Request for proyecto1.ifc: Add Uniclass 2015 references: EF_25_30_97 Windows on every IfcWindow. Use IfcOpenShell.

First a look at what the model holds.

```python
import ifcopenshell

model = ifcopenshell.open("proyecto1.ifc")
print(model.schema)
print("classifications:", [c.Name for c in model.by_type("IfcClassification")])
for ifc_class in ("IfcDoor", "IfcRoof", "IfcStair", "IfcWall", "IfcWindow"):
    print(ifc_class, len(model.by_type(ifc_class)))
```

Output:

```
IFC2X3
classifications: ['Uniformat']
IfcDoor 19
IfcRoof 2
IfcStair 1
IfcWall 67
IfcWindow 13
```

```python
import ifcopenshell
import ifcopenshell.api.classification

model = ifcopenshell.open("proyecto1.ifc")

# IFC2X3 requires Source and Edition and has no link from the project to the system.
system = model.create_entity("IfcClassification", Source="NBS", Edition="2015", Name="Uniclass 2015")

codes = {
    "IfcWindow": ("EF_25_30_97", "Windows"),
}
for ifc_class, (code, name) in codes.items():
    products = model.by_type(ifc_class)
    ifcopenshell.api.classification.add_reference(
        model, products=products, classification=system, identification=code, name=name
    )
    print(code, len(products))

model.write("proyecto1_edited.ifc")
```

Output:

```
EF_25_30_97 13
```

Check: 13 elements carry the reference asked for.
